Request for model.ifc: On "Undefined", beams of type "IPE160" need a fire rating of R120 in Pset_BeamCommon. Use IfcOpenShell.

First a look at what the model holds.

```python
import ifcopenshell
import ifcopenshell.util.element

model = ifcopenshell.open("model.ifc")
print(model.schema)
storey = next(s for s in model.by_type("IfcBuildingStorey") if s.Name == "Undefined")
beams = [e for e in ifcopenshell.util.element.get_decomposition(storey) if e.is_a("IfcBeam")]
seen = {}
for e in beams:
    element_type = ifcopenshell.util.element.get_type(e)
    key = (element_type.Name if element_type != e and element_type else None, ifcopenshell.util.element.get_pset(e, "Pset_BeamCommon", "FireRating"))
    seen[key] = seen.get(key, 0) + 1
for (name, value), count in sorted(seen.items(), key=str):
    print(count, "x", name, "|", value)
```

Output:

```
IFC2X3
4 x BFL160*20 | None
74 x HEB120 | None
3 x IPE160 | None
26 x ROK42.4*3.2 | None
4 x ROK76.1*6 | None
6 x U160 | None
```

```python
import ifcopenshell
import ifcopenshell.api.pset
import ifcopenshell.util.element

model = ifcopenshell.open("model.ifc")

storey = next(s for s in model.by_type("IfcBuildingStorey") if s.Name == "Undefined")
beams = [e for e in ifcopenshell.util.element.get_decomposition(storey) if e.is_a("IfcBeam")]

count = 0
for e in beams:
    element_type = ifcopenshell.util.element.get_type(e)
    if element_type in (None, e) or element_type.Name != "IPE160":
        continue
    # add_pset returns the element's existing set when there is one.
    pset = ifcopenshell.api.pset.add_pset(model, product=e, name="Pset_BeamCommon")
    ifcopenshell.api.pset.edit_pset(model, pset=pset, properties={"FireRating": "R120"})
    count += 1

print(count, "beams updated")

model.write("model_updated.ifc")
```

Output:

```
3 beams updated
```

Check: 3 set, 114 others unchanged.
